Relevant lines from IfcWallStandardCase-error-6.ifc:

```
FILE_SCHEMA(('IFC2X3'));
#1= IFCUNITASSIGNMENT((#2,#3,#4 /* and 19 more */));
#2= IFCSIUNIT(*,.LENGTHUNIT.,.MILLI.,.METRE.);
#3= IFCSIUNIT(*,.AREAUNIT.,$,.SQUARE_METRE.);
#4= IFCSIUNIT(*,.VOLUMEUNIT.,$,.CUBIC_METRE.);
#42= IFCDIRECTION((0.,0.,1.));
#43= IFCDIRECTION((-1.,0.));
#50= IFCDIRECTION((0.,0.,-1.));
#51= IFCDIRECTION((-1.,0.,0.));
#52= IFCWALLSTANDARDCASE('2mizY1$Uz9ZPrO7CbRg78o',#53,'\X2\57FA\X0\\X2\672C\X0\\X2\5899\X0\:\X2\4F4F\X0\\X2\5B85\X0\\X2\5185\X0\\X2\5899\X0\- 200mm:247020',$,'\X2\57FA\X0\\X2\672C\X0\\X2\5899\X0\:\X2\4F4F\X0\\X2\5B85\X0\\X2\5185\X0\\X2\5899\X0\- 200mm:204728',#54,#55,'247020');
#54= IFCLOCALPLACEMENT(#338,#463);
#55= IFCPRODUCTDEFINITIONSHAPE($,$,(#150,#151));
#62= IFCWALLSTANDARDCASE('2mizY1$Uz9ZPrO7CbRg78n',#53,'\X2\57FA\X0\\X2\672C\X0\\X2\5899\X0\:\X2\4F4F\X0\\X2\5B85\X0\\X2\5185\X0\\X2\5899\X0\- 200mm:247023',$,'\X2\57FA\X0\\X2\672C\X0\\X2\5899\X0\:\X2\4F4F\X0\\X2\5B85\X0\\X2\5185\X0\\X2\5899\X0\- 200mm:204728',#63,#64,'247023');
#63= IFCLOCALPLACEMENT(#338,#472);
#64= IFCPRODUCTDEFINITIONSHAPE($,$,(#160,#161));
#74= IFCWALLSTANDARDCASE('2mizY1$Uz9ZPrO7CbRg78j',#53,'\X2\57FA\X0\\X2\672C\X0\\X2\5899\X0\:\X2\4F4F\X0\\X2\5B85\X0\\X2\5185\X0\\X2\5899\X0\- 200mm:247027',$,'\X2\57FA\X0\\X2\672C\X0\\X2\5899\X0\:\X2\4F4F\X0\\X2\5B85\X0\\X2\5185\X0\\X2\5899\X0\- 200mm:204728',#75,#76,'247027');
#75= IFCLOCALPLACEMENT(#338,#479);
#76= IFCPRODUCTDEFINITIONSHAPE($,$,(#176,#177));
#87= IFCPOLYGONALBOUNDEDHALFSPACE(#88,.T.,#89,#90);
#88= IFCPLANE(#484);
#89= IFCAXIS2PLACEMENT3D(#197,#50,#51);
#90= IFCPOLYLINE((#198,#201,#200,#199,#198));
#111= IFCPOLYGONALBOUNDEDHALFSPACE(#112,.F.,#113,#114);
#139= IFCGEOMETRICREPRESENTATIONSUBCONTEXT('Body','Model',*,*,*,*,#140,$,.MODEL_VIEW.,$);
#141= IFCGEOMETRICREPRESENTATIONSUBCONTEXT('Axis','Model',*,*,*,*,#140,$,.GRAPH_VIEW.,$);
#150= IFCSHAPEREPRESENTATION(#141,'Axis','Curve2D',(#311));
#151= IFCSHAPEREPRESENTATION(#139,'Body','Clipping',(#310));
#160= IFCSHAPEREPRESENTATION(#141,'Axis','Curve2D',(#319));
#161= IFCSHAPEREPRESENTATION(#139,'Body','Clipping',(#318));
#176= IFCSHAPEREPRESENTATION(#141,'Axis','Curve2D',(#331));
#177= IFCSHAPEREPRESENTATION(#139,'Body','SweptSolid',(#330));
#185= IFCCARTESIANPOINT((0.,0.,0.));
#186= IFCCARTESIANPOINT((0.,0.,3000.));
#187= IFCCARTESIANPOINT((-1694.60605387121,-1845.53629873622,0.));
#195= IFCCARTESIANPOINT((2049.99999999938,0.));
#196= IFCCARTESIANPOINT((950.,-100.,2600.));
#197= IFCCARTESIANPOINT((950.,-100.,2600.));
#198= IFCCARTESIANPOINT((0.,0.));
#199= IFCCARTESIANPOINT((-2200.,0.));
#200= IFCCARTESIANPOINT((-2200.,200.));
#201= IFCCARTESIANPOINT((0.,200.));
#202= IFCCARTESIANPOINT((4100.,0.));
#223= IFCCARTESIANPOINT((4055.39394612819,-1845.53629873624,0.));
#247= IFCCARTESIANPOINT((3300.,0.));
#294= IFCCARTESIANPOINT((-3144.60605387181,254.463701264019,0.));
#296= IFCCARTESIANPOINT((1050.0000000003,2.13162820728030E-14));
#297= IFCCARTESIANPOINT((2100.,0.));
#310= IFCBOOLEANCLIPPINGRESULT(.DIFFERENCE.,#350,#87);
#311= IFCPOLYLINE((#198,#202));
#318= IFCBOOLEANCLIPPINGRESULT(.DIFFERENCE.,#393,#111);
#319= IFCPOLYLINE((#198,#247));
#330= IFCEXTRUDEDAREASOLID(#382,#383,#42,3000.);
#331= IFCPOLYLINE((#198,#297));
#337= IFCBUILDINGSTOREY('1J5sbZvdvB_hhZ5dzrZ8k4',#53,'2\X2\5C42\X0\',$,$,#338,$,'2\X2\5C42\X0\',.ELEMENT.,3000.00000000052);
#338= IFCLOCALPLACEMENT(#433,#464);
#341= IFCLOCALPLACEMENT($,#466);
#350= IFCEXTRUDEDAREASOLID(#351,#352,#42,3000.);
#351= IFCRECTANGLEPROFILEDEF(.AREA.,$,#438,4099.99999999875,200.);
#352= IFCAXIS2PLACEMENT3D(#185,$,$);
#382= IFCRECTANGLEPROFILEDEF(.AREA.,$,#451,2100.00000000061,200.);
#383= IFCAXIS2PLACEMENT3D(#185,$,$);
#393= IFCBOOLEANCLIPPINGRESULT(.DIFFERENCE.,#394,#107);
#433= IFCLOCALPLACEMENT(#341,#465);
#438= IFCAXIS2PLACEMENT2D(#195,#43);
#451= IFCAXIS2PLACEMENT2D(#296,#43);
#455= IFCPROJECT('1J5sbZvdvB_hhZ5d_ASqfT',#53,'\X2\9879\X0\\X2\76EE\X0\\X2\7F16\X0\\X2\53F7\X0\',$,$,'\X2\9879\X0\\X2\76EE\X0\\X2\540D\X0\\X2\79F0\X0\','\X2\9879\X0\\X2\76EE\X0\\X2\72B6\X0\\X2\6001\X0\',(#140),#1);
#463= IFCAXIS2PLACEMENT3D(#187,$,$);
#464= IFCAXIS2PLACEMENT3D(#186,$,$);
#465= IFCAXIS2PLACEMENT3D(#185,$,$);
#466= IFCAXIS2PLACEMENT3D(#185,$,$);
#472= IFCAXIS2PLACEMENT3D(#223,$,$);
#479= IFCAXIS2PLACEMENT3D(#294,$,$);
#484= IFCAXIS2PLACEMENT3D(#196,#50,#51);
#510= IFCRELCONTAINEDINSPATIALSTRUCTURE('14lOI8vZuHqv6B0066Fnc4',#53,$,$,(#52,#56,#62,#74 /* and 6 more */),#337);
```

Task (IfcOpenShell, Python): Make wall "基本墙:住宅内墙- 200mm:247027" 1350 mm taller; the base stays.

```python
import ifcopenshell
import ifcopenshell.geom
import ifcopenshell.util.representation
import ifcopenshell.util.shape
import ifcopenshell.util.unit

model = ifcopenshell.open("IfcWallStandardCase-error-6.ifc")
unit_scale = ifcopenshell.util.unit.calculate_unit_scale(model)
settings = ifcopenshell.geom.settings()


def volume(element):
    """Net volume in cubic metres, openings subtracted."""
    shape = ifcopenshell.geom.create_shape(settings, element)
    return ifcopenshell.util.shape.get_volume(shape.geometry)


wall = model.by_guid("2mizY1$Uz9ZPrO7CbRg78j")
before = volume(wall)

body = ifcopenshell.util.representation.get_representation(wall, "Model", "Body")
solid = body.Items[0]
old_height = solid.Depth
solid.Depth += 1.35 / unit_scale
after = volume(wall)

print(f"height {old_height:g} -> {solid.Depth:g}, volume {before:.3f} -> {after:.3f} m3")

model.write("IfcWallStandardCase-error-6_v2.ifc")
```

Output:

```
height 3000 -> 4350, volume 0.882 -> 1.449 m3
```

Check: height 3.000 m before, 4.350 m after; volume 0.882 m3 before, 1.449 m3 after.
